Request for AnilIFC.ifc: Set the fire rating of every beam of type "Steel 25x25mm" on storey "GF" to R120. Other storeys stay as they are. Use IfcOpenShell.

First a look at what the model holds.

```python
import ifcopenshell
import ifcopenshell.util.element

model = ifcopenshell.open("AnilIFC.ifc")
print(model.schema)
storey = next(s for s in model.by_type("IfcBuildingStorey") if s.Name == "GF")
beams = [e for e in ifcopenshell.util.element.get_decomposition(storey) if e.is_a("IfcBeam")]
seen = {}
for e in beams:
    element_type = ifcopenshell.util.element.get_type(e)
    key = (element_type.Name if element_type != e and element_type else None, ifcopenshell.util.element.get_pset(e, "Pset_BeamCommon", "FireRating"))
    seen[key] = seen.get(key, 0) + 1
for (name, value), count in sorted(seen.items(), key=str):
    print(count, "x", name, "|", value)
```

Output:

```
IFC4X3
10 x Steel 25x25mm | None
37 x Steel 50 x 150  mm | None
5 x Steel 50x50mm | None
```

```python
import ifcopenshell
import ifcopenshell.api.pset
import ifcopenshell.util.element

model = ifcopenshell.open("AnilIFC.ifc")

storey = next(s for s in model.by_type("IfcBuildingStorey") if s.Name == "GF")
beams = [e for e in ifcopenshell.util.element.get_decomposition(storey) if e.is_a("IfcBeam")]

count = 0
for e in beams:
    element_type = ifcopenshell.util.element.get_type(e)
    if element_type in (None, e) or element_type.Name != "Steel 25x25mm":
        continue
    # add_pset returns the element's existing set when there is one.
    pset = ifcopenshell.api.pset.add_pset(model, product=e, name="Pset_BeamCommon")
    ifcopenshell.api.pset.edit_pset(model, pset=pset, properties={"FireRating": "R120"})
    count += 1

print(count, "beams updated")

model.write("AnilIFC_updated.ifc")
```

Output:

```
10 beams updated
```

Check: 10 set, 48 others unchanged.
